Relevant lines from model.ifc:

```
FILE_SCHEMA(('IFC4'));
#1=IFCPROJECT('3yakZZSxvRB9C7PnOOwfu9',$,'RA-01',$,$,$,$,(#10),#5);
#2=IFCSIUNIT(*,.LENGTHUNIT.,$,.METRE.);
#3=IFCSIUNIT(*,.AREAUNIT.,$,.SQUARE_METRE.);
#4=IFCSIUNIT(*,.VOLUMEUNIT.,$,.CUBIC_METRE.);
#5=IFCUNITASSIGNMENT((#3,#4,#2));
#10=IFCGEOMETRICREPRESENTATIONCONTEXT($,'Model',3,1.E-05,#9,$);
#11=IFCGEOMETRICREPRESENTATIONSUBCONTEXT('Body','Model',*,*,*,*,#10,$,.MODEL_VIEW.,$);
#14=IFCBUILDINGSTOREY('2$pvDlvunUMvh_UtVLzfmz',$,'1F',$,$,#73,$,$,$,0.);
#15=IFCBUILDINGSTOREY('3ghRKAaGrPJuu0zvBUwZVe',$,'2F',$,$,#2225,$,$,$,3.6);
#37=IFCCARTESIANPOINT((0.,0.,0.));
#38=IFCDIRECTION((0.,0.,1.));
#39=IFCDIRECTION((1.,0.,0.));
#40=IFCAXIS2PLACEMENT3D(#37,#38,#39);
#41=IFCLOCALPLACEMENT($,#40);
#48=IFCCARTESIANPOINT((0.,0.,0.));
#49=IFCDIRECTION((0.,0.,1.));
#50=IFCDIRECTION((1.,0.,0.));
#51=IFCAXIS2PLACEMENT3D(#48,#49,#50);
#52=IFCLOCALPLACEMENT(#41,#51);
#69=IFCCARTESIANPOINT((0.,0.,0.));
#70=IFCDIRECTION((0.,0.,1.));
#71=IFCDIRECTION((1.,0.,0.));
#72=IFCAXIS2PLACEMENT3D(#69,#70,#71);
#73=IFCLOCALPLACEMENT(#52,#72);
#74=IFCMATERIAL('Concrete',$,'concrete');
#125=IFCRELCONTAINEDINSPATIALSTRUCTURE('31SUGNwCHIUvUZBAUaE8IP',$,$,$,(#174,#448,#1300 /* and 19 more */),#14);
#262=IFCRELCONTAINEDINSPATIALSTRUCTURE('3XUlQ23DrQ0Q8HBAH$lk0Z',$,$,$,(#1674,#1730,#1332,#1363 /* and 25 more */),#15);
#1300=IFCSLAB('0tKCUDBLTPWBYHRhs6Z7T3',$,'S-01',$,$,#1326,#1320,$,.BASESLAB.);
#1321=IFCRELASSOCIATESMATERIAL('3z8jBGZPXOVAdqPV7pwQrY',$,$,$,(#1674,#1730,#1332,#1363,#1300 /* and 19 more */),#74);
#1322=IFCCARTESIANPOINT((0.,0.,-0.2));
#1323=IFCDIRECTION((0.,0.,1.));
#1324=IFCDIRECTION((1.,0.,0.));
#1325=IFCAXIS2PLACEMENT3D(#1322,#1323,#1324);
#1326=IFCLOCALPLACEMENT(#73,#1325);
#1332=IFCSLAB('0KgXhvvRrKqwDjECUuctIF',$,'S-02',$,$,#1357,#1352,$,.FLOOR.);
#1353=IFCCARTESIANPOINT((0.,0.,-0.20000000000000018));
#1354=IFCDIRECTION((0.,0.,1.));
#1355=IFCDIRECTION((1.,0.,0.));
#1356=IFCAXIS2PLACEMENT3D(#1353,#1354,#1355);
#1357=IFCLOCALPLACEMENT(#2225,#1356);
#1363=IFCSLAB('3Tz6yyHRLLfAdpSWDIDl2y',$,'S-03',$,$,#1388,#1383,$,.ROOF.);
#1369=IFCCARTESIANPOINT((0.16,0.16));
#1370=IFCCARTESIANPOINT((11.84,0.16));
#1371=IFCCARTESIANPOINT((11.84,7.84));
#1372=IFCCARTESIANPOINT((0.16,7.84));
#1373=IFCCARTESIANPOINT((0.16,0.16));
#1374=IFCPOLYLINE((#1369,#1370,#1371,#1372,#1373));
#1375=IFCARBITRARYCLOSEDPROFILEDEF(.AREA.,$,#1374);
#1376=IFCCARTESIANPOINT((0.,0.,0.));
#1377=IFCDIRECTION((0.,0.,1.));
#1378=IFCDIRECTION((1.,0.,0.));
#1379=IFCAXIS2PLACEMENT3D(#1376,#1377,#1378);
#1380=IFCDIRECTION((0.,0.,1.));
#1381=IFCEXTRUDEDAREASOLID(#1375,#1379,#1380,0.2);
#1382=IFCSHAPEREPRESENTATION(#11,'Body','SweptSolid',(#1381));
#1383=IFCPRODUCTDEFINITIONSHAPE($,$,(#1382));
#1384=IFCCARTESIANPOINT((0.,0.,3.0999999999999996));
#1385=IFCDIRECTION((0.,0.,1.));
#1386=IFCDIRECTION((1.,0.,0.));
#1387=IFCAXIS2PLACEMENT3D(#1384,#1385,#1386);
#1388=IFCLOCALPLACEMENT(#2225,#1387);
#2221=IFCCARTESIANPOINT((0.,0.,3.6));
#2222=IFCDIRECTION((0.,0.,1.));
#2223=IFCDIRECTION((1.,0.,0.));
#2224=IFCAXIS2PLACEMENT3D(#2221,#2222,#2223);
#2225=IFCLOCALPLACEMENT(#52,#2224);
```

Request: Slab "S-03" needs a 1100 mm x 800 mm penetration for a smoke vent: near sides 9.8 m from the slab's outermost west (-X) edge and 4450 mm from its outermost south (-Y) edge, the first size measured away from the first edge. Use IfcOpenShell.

```python
import numpy as np
import ifcopenshell
import ifcopenshell.api.feature
import ifcopenshell.api.geometry
import ifcopenshell.api.root
import ifcopenshell.geom
import ifcopenshell.util.placement
import ifcopenshell.util.representation
import ifcopenshell.util.shape
import ifcopenshell.util.unit

model = ifcopenshell.open("model.ifc")
unit_scale = ifcopenshell.util.unit.calculate_unit_scale(model)
settings = ifcopenshell.geom.settings()


def volume(element):
    """Net volume in cubic metres, openings subtracted."""
    shape = ifcopenshell.geom.create_shape(settings, element)
    return ifcopenshell.util.shape.get_volume(shape.geometry)


slab = model.by_guid("3Tz6yyHRLLfAdpSWDIDl2y")
before = volume(slab)

# Extent in the slab's own axes, in metres. The edges named are its -X and -Y sides.
slab_shape = ifcopenshell.geom.create_shape(settings, slab)
vertices = ifcopenshell.util.shape.get_vertices(slab_shape.geometry)
x_min, y_min, bottom = vertices.min(axis=0)
top = vertices[:, 2].max()

opening = ifcopenshell.api.root.create_entity(model, ifc_class="IfcOpeningElement", name="Smoke vent opening", predefined_type="OPENING")
context = ifcopenshell.util.representation.get_context(model, "Model", "Body", "MODEL_VIEW")
width, depth = 1.1, 0.8
outline = [(0.0, 0.0), (width, 0.0), (width, depth), (0.0, depth), (0.0, 0.0)]
# Overshoot both faces by 50 mm so the cut is clean.
shape = ifcopenshell.api.geometry.add_slab_representation(
    model, context=context, depth=top - bottom + 0.1, polyline=outline
)
ifcopenshell.api.geometry.assign_representation(model, product=opening, representation=shape)

matrix = ifcopenshell.util.placement.get_local_placement(slab.ObjectPlacement)
matrix[:, 3] = matrix @ np.append(np.array([x_min + 9.8, y_min + 4.45, bottom - 0.05]) / unit_scale, 1.0)
ifcopenshell.api.geometry.edit_object_placement(model, product=opening, matrix=matrix, is_si=False)
ifcopenshell.api.feature.add_feature(model, feature=opening, element=slab)

after = volume(slab)

print(f"slab volume {before:.3f} -> {after:.3f} m3")

model.write("model_edited.ifc")
```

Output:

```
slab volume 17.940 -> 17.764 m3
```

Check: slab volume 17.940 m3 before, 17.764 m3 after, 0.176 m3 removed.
